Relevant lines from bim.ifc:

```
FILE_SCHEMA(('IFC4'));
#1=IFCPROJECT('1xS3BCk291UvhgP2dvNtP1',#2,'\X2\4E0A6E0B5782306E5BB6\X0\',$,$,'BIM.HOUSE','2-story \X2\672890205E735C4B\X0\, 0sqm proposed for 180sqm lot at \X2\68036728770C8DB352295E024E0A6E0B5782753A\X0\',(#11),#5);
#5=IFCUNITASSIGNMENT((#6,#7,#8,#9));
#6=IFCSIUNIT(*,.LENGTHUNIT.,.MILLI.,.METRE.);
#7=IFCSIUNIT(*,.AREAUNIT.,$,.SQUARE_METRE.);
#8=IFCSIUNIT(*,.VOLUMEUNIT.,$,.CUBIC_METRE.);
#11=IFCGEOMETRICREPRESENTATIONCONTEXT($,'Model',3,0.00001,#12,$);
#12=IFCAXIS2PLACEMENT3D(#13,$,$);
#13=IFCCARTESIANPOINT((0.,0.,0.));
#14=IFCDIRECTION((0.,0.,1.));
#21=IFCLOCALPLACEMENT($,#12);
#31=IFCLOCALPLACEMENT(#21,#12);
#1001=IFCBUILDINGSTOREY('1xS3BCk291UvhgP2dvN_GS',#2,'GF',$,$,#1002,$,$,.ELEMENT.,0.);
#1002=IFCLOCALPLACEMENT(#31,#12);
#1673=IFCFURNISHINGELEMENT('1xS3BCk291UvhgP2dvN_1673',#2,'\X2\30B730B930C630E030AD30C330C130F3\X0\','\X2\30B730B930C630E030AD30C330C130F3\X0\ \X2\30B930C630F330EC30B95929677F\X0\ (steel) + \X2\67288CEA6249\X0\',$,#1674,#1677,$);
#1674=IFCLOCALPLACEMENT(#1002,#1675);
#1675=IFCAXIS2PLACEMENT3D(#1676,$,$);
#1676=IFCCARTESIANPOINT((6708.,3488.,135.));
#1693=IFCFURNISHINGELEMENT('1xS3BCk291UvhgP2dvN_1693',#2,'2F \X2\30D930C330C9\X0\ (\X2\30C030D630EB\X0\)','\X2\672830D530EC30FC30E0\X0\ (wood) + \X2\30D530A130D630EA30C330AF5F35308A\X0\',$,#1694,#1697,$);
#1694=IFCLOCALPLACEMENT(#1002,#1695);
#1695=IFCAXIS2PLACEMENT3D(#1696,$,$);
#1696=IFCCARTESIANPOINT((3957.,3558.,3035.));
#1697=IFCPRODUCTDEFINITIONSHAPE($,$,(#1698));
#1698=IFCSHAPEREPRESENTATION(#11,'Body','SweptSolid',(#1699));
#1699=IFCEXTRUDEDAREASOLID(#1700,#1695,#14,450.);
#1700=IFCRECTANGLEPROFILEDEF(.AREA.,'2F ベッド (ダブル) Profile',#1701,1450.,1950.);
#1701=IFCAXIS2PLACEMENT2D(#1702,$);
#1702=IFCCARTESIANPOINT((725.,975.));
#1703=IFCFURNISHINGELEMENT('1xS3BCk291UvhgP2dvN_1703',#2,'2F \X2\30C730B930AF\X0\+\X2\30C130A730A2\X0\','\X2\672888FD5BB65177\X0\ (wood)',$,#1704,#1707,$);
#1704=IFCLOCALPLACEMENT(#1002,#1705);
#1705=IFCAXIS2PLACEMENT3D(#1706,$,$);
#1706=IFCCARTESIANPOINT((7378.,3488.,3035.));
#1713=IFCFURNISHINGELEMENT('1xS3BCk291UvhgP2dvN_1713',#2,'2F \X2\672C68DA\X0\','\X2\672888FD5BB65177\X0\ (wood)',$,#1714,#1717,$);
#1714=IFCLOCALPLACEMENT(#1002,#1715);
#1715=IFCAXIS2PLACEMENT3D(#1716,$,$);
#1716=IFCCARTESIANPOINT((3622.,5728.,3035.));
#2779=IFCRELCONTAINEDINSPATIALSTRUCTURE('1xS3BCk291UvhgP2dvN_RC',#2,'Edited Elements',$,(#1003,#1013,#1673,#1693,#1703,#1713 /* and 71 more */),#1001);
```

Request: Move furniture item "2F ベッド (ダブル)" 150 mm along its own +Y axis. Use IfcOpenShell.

```python
import ifcopenshell
import ifcopenshell.api.geometry
import ifcopenshell.util.placement
import ifcopenshell.util.unit

model = ifcopenshell.open("bim.ifc")
unit_scale = ifcopenshell.util.unit.calculate_unit_scale(model)

item = model.by_id(1693)
matrix = ifcopenshell.util.placement.get_local_placement(item.ObjectPlacement)
matrix[:3, 3] += matrix[:3, 1] * 0.15 / unit_scale
ifcopenshell.api.geometry.edit_object_placement(model, product=item, matrix=matrix, is_si=False)

print(ifcopenshell.util.placement.get_local_placement(item.ObjectPlacement).round(3) + 0.0)

model.write("bim_edited.ifc")
```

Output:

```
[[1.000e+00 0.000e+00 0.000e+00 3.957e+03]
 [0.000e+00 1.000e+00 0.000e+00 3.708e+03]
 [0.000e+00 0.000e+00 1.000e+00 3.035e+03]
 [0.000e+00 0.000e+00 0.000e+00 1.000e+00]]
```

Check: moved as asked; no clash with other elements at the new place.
